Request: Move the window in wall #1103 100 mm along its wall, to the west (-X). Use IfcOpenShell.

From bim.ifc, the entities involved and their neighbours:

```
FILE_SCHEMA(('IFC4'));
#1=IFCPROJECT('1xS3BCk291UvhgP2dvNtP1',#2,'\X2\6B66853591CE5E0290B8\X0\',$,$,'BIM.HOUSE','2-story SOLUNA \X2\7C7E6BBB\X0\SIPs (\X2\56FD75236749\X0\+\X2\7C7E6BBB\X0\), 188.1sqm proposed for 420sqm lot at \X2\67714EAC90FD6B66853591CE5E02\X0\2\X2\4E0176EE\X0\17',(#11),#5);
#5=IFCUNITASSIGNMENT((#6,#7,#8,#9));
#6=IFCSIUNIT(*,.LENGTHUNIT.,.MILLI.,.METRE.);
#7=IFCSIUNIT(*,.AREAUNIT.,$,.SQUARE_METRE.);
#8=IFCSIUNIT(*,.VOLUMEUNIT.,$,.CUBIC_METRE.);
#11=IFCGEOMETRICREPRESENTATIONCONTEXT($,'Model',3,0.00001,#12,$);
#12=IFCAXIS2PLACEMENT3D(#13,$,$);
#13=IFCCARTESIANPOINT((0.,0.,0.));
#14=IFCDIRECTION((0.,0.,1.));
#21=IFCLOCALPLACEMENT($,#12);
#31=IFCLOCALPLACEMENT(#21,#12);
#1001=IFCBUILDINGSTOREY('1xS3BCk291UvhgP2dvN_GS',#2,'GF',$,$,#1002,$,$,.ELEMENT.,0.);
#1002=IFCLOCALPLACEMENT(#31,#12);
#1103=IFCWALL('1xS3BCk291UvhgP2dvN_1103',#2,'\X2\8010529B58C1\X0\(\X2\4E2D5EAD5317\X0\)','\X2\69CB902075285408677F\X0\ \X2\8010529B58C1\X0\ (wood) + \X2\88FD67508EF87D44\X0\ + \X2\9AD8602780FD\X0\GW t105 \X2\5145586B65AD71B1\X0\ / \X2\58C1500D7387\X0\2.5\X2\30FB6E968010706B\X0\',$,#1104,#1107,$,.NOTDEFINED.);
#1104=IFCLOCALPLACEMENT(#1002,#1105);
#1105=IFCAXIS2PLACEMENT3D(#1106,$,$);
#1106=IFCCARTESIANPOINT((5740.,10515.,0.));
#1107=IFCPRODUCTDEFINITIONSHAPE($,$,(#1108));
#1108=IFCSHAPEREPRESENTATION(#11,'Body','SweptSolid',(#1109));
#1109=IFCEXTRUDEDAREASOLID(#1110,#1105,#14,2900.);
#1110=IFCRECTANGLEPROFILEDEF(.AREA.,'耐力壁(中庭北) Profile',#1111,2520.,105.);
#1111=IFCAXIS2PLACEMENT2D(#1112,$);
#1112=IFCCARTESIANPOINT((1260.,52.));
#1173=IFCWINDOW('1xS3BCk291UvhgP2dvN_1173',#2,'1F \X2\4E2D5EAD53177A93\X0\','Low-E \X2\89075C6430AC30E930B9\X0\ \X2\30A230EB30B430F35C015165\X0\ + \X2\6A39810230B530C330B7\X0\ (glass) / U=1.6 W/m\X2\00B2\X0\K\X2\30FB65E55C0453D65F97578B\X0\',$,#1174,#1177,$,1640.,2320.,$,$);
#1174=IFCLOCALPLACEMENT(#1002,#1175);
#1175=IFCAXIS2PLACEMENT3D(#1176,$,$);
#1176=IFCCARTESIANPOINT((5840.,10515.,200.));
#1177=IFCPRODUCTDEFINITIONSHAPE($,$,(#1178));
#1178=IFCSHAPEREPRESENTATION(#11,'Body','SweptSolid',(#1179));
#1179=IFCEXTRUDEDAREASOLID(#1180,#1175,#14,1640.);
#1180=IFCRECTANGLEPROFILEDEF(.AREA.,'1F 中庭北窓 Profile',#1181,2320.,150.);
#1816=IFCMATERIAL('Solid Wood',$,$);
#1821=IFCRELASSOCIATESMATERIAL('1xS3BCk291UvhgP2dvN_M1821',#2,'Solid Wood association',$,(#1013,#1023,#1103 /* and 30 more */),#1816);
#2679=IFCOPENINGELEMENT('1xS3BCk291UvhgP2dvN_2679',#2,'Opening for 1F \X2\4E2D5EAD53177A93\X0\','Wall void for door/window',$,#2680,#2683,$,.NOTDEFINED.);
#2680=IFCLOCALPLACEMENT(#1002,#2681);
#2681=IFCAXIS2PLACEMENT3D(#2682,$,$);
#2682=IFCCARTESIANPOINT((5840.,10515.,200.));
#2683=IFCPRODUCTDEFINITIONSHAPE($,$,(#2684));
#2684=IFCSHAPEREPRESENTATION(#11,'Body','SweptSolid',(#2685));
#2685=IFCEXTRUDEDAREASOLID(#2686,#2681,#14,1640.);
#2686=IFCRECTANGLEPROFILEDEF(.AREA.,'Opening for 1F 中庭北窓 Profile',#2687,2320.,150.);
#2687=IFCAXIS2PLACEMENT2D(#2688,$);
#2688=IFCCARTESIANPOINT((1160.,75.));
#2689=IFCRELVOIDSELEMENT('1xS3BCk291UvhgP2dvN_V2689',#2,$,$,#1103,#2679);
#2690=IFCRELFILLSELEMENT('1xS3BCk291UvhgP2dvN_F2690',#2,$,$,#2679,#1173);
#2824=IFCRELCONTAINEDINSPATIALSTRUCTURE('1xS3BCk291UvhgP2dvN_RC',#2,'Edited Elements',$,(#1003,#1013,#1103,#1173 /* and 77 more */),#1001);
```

```python
import ifcopenshell
import ifcopenshell.api.geometry
import ifcopenshell.util.placement

model = ifcopenshell.open("bim.ifc")

window = model.by_guid("1xS3BCk291UvhgP2dvN_1173")
opening = window.FillsVoids[0].RelatingOpeningElement
wall = opening.VoidsElements[0].RelatingBuildingElement

wall_matrix = ifcopenshell.util.placement.get_local_placement(wall.ObjectPlacement)
shift = wall_matrix[:3, 0] * -100.0
before = ifcopenshell.util.placement.get_local_placement(window.ObjectPlacement)[:3, 3].copy()

# The window is not placed relative to its opening, so move both.
for product in (opening, window):
    matrix = ifcopenshell.util.placement.get_local_placement(product.ObjectPlacement)
    matrix[:3, 3] += shift
    ifcopenshell.api.geometry.edit_object_placement(model, product=product, matrix=matrix, is_si=False)

after = ifcopenshell.util.placement.get_local_placement(window.ObjectPlacement)[:3, 3]
print("window moved by", (after - before).round(3) + 0.0)

model.write("bim-out.ifc")
```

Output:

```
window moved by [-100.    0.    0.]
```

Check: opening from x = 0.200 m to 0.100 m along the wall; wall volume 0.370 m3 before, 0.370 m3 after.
